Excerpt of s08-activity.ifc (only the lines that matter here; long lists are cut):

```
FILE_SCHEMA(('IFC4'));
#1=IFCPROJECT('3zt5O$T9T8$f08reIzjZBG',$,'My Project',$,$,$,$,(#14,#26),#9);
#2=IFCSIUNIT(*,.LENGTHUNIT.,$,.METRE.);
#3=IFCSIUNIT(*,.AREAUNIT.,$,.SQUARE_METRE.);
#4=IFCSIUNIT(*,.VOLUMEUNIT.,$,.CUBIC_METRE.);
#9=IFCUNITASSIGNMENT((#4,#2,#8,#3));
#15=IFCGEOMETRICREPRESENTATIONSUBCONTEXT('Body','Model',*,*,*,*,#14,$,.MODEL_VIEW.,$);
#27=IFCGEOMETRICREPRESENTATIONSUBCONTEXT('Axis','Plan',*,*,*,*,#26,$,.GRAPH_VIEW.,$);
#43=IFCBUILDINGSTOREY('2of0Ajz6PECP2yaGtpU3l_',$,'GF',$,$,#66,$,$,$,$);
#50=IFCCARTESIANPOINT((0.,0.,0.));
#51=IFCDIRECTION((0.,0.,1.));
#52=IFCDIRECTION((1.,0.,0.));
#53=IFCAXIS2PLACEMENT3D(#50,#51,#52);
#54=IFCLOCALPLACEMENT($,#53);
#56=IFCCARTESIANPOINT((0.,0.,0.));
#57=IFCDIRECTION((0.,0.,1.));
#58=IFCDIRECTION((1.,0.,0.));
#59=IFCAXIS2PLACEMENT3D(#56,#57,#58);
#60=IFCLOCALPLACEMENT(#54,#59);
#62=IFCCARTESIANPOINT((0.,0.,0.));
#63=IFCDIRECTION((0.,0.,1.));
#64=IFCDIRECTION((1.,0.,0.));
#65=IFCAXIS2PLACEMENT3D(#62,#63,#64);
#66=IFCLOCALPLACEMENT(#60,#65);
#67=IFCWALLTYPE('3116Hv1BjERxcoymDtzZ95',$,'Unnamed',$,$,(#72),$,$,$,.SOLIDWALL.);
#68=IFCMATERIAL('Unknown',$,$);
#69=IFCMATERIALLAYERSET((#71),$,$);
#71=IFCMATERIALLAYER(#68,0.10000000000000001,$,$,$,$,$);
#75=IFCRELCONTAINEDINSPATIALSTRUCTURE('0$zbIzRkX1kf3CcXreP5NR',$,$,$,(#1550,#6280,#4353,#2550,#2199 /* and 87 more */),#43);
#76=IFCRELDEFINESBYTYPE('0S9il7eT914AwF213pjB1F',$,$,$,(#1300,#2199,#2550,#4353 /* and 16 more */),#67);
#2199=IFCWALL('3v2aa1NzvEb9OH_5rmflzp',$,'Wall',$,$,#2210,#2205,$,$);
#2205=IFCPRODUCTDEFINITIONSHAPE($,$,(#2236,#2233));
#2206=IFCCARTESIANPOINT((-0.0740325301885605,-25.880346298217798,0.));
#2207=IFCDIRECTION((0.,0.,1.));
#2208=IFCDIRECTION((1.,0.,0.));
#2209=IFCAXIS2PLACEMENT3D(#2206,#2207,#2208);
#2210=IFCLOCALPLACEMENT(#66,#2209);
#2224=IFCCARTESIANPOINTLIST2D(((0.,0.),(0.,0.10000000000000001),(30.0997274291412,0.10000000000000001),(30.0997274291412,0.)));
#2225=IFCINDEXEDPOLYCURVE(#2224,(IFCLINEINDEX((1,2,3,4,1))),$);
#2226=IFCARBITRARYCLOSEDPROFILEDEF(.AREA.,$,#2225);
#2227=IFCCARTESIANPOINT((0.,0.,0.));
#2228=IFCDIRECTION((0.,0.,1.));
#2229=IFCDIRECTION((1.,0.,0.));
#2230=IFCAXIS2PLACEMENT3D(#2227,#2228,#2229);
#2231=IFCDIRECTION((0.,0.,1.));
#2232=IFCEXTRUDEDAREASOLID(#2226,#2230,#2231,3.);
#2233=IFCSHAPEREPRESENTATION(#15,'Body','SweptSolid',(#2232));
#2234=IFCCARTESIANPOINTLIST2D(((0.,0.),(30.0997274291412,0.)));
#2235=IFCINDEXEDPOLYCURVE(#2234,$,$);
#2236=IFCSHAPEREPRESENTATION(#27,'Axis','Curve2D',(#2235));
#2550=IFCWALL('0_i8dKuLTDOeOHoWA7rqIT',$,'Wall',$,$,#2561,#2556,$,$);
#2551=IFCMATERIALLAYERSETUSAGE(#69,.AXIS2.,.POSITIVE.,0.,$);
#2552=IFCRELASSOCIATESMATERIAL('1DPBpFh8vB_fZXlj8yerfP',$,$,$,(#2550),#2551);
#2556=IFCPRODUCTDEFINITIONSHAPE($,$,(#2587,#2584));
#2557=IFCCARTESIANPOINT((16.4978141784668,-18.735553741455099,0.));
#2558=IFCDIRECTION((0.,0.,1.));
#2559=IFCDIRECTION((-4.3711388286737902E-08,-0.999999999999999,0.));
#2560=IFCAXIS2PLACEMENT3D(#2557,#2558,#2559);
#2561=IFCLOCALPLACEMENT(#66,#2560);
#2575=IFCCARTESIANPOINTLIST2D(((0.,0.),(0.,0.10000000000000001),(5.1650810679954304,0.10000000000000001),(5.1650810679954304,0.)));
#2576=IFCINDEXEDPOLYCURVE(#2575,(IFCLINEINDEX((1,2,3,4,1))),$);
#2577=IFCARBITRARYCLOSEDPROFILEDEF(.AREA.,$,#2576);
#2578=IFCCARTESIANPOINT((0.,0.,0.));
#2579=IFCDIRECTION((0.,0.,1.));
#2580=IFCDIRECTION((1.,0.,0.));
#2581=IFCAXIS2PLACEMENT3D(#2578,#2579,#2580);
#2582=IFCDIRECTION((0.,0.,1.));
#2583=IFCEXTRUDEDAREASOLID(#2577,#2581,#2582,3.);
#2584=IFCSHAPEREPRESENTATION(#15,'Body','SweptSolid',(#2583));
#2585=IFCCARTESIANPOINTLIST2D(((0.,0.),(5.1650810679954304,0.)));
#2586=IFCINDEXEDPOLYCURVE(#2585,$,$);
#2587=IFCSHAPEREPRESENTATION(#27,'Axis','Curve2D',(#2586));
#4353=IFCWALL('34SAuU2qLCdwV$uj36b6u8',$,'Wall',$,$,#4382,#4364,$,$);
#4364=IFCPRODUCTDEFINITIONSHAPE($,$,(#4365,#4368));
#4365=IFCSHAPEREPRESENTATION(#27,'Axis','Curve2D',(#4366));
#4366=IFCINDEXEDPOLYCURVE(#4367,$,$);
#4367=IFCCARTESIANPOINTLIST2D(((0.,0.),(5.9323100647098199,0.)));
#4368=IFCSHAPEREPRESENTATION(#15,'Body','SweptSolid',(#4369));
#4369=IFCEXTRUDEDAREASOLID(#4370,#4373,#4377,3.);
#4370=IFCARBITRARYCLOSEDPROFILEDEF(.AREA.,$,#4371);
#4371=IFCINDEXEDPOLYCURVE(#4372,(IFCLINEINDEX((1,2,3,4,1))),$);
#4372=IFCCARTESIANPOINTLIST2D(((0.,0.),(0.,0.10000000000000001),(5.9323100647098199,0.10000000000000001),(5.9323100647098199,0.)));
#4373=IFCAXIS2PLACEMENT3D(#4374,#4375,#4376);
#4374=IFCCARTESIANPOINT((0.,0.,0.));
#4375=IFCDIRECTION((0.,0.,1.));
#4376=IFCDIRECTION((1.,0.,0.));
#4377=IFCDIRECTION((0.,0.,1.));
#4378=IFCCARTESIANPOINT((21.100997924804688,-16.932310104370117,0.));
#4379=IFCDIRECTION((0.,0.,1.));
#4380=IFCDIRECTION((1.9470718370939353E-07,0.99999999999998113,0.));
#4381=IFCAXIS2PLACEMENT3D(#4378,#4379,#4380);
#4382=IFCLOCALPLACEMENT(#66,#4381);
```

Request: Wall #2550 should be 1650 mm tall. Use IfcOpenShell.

```python
import ifcopenshell
import ifcopenshell.geom
import ifcopenshell.util.representation
import ifcopenshell.util.shape
import ifcopenshell.util.unit

model = ifcopenshell.open("s08-activity.ifc")
unit_scale = ifcopenshell.util.unit.calculate_unit_scale(model)
settings = ifcopenshell.geom.settings()


def volume(element):
    """Net volume in cubic metres, openings subtracted."""
    shape = ifcopenshell.geom.create_shape(settings, element)
    return ifcopenshell.util.shape.get_volume(shape.geometry)


wall = model.by_guid("0_i8dKuLTDOeOHoWA7rqIT")
before = volume(wall)

body = ifcopenshell.util.representation.get_representation(wall, "Model", "Body")
solid = body.Items[0]
old_height = solid.Depth
solid.Depth = 1.65 / unit_scale
after = volume(wall)

print(f"height {old_height:g} -> {solid.Depth:g}, volume {before:.3f} -> {after:.3f} m3")

model.write("s08-activity_updated.ifc")
```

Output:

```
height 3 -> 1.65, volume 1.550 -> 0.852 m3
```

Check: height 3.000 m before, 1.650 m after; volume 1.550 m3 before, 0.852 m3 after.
